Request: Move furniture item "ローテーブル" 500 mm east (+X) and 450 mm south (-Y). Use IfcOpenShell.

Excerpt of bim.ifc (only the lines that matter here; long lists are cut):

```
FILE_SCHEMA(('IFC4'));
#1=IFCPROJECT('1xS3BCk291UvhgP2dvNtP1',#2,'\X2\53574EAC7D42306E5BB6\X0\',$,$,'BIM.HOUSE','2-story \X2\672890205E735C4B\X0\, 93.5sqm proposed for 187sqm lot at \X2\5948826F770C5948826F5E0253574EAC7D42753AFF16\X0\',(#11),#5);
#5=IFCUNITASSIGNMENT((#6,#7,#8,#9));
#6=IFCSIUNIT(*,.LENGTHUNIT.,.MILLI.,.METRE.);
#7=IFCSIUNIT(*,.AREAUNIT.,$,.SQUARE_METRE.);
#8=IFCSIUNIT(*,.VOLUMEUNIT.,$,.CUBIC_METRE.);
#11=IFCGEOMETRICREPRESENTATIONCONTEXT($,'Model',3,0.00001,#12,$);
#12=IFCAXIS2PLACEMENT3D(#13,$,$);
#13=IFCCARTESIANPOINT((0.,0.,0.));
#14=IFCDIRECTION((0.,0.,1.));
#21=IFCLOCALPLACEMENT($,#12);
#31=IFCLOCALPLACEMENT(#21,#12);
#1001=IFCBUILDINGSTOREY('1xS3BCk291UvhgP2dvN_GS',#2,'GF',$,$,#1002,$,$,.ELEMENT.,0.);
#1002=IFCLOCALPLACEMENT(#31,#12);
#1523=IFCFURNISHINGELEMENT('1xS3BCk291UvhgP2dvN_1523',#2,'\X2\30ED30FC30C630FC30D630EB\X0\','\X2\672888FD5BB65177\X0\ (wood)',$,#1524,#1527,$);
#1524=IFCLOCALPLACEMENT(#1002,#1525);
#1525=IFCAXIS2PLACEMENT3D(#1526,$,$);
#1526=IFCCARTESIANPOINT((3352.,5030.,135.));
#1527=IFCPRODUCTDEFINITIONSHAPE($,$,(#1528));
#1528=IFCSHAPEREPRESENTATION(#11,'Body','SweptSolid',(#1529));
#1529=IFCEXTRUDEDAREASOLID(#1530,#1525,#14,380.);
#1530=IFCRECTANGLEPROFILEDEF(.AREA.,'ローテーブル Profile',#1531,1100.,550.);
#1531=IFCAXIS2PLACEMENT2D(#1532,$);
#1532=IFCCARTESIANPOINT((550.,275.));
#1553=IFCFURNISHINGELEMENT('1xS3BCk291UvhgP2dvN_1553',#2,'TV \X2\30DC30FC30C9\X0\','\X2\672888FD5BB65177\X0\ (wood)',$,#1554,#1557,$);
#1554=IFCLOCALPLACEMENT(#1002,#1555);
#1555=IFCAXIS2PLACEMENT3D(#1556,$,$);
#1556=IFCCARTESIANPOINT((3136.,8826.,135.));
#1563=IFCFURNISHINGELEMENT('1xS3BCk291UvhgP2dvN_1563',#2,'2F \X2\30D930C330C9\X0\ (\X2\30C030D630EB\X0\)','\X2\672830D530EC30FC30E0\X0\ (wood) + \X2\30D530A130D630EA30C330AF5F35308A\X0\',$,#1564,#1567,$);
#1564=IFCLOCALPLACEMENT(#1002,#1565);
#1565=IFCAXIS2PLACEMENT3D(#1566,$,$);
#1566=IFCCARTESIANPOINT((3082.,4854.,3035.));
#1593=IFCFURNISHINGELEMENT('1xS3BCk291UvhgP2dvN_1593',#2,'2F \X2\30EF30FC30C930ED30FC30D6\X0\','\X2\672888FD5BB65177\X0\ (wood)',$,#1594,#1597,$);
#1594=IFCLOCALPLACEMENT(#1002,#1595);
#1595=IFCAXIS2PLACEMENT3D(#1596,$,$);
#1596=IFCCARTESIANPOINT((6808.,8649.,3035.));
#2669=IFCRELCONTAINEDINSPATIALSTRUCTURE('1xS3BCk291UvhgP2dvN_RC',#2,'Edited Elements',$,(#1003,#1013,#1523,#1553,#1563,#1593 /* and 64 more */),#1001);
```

```python
import ifcopenshell
import ifcopenshell.api.geometry
import ifcopenshell.util.placement
import ifcopenshell.util.unit

model = ifcopenshell.open("bim.ifc")
unit_scale = ifcopenshell.util.unit.calculate_unit_scale(model)

item = model.by_id(1523)
matrix = ifcopenshell.util.placement.get_local_placement(item.ObjectPlacement)
matrix[0, 3] += 0.5 / unit_scale
matrix[1, 3] -= 0.45 / unit_scale
ifcopenshell.api.geometry.edit_object_placement(model, product=item, matrix=matrix, is_si=False)

print(ifcopenshell.util.placement.get_local_placement(item.ObjectPlacement).round(3) + 0.0)

model.write("bim_updated.ifc")
```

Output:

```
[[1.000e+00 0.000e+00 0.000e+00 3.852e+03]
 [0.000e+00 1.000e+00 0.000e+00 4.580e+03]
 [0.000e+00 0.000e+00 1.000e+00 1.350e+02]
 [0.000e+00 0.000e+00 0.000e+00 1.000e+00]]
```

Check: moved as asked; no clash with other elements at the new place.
